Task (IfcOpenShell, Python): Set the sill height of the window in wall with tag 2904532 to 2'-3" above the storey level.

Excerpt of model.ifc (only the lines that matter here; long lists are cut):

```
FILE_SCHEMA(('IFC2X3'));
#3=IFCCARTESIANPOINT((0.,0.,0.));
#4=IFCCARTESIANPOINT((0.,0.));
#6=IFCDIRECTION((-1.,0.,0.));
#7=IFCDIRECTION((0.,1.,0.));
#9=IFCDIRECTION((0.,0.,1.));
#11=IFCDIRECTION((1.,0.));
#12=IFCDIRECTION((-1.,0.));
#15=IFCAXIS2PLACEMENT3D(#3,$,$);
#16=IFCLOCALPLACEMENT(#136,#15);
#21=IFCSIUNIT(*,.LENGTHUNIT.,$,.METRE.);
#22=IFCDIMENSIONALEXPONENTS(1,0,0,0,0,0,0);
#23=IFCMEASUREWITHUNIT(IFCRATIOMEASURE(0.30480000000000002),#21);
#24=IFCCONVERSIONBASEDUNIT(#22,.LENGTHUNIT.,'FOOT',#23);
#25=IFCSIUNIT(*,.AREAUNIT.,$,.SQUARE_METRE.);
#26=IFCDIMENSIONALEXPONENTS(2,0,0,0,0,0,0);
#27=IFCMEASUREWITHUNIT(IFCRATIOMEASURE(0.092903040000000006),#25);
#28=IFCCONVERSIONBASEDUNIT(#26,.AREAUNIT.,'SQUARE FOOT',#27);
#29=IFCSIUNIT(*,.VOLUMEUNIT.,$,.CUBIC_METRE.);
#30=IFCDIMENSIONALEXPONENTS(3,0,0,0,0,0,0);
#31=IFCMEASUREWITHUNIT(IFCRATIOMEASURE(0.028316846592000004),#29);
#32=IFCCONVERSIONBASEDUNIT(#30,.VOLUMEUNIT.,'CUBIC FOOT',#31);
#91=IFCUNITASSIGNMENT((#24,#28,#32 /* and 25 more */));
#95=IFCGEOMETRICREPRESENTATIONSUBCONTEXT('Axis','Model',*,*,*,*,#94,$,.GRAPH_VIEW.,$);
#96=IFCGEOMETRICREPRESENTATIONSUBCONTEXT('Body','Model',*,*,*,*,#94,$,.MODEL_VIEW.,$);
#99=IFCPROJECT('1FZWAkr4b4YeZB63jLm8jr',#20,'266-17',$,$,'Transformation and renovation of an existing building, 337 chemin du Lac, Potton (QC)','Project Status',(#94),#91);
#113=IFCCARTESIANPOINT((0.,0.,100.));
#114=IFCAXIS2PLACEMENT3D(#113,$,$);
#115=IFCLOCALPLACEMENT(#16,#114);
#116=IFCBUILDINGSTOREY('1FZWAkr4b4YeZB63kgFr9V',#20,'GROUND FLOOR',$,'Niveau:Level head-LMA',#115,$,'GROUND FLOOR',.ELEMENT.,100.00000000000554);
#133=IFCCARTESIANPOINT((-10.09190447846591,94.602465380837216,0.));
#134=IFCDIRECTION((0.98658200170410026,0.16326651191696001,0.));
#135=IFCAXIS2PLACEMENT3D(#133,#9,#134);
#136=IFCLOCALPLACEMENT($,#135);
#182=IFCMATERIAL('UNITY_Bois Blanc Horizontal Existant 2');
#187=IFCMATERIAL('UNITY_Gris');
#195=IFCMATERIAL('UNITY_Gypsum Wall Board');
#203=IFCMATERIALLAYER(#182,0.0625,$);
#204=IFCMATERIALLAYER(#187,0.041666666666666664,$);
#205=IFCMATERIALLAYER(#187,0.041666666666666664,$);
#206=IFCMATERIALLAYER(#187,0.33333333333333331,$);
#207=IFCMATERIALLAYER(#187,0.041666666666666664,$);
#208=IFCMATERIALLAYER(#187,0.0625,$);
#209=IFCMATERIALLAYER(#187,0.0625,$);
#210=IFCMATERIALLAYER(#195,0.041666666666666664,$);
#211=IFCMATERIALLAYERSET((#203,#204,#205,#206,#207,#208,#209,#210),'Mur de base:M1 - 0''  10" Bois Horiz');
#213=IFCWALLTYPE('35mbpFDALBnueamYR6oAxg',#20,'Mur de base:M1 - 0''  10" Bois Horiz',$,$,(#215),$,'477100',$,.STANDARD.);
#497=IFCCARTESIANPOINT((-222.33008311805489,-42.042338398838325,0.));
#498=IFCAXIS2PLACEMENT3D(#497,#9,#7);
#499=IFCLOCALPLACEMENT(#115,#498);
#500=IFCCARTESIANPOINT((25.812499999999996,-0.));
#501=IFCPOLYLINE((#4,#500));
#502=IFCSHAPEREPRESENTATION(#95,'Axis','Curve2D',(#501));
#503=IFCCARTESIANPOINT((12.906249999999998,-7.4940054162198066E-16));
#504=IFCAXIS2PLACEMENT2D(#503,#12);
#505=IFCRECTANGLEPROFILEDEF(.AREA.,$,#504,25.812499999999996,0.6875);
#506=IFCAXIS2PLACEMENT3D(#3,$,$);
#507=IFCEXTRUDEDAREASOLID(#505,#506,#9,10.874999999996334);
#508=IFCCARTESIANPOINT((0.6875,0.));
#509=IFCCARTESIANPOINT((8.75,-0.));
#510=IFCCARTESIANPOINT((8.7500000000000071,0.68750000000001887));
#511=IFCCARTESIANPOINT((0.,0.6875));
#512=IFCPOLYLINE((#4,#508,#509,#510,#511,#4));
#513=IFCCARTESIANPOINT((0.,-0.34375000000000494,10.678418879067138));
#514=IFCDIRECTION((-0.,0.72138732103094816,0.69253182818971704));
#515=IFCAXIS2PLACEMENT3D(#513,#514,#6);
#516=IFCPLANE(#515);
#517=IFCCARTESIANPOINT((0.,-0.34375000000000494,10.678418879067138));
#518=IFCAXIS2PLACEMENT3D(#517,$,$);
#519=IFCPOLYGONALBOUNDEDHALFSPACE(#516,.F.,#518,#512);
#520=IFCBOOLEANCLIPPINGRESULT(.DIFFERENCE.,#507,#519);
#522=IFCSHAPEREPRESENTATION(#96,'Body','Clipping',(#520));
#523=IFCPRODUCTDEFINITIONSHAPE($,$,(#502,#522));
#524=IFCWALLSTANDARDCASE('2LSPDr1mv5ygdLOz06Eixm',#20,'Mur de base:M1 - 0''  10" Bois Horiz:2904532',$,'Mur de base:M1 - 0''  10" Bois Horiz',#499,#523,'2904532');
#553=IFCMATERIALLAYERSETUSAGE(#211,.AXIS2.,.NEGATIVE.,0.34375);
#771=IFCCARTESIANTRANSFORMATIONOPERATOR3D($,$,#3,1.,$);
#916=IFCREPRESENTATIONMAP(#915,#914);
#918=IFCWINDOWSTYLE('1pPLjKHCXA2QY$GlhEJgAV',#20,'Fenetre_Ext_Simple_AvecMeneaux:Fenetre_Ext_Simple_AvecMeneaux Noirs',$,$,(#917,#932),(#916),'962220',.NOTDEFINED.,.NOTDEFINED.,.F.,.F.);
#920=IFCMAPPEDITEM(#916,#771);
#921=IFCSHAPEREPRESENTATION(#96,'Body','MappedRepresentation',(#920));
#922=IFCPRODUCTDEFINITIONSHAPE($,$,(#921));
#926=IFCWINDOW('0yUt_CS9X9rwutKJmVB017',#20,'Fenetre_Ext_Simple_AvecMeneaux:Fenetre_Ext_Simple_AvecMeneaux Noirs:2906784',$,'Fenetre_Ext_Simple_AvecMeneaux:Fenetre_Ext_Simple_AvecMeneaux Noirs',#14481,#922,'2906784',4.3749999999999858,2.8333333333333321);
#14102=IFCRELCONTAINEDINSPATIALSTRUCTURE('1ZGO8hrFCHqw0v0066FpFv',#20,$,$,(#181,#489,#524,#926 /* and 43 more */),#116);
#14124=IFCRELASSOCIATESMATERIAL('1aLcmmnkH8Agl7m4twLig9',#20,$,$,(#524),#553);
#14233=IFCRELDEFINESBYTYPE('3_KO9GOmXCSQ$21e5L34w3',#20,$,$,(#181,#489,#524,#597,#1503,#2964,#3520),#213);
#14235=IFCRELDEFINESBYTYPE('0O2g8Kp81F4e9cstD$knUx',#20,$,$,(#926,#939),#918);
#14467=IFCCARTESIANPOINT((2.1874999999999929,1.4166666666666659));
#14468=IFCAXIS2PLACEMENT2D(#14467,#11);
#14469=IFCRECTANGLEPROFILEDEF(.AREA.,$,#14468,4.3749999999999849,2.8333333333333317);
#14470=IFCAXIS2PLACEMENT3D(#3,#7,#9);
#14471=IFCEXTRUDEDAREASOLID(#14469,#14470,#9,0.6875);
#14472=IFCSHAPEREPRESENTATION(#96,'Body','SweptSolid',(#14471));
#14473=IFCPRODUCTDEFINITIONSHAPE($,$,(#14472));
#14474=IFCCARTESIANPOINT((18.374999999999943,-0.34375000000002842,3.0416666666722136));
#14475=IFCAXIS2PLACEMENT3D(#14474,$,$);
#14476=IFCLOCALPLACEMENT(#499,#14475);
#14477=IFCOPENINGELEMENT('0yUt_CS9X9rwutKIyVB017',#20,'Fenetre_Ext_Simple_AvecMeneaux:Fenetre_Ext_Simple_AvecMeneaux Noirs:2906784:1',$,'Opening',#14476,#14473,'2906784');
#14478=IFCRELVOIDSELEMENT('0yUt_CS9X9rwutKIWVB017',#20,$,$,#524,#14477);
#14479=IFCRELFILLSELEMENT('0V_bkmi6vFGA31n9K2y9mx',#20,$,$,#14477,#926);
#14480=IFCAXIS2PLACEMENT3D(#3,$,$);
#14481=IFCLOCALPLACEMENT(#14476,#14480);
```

```python
import numpy as np
import ifcopenshell
import ifcopenshell.api.geometry
import ifcopenshell.geom
import ifcopenshell.util.element
import ifcopenshell.util.placement
import ifcopenshell.util.shape
import ifcopenshell.util.unit

model = ifcopenshell.open("model.ifc")
unit_scale = ifcopenshell.util.unit.calculate_unit_scale(model)

window = model.by_id(926)
opening = window.FillsVoids[0].RelatingOpeningElement
storey = ifcopenshell.util.element.get_container(window, ifc_class="IfcBuildingStorey")
level = ifcopenshell.util.placement.get_local_placement(storey.ObjectPlacement)[2, 3]

# The opening's origin need not be at the sill, so measure its lowest point.
shape = ifcopenshell.geom.create_shape(ifcopenshell.geom.settings(), opening)
bottom = ifcopenshell.util.shape.get_shape_bottom_elevation(shape, shape.geometry) / unit_scale
dz = level + 27 * 0.0254 / unit_scale - bottom

shift = np.array([0.0, 0.0, dz])
# The window is placed relative to its opening, so it follows when the opening moves.
matrix = ifcopenshell.util.placement.get_local_placement(opening.ObjectPlacement)
matrix[:3, 3] += shift
ifcopenshell.api.geometry.edit_object_placement(
    model, product=opening, matrix=matrix, is_si=False, should_transform_children=True
)

print(f"moved by {dz * unit_scale:+.3f} m")

model.write("model_v2.ifc")
```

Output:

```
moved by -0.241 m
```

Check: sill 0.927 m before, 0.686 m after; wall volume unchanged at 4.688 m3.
